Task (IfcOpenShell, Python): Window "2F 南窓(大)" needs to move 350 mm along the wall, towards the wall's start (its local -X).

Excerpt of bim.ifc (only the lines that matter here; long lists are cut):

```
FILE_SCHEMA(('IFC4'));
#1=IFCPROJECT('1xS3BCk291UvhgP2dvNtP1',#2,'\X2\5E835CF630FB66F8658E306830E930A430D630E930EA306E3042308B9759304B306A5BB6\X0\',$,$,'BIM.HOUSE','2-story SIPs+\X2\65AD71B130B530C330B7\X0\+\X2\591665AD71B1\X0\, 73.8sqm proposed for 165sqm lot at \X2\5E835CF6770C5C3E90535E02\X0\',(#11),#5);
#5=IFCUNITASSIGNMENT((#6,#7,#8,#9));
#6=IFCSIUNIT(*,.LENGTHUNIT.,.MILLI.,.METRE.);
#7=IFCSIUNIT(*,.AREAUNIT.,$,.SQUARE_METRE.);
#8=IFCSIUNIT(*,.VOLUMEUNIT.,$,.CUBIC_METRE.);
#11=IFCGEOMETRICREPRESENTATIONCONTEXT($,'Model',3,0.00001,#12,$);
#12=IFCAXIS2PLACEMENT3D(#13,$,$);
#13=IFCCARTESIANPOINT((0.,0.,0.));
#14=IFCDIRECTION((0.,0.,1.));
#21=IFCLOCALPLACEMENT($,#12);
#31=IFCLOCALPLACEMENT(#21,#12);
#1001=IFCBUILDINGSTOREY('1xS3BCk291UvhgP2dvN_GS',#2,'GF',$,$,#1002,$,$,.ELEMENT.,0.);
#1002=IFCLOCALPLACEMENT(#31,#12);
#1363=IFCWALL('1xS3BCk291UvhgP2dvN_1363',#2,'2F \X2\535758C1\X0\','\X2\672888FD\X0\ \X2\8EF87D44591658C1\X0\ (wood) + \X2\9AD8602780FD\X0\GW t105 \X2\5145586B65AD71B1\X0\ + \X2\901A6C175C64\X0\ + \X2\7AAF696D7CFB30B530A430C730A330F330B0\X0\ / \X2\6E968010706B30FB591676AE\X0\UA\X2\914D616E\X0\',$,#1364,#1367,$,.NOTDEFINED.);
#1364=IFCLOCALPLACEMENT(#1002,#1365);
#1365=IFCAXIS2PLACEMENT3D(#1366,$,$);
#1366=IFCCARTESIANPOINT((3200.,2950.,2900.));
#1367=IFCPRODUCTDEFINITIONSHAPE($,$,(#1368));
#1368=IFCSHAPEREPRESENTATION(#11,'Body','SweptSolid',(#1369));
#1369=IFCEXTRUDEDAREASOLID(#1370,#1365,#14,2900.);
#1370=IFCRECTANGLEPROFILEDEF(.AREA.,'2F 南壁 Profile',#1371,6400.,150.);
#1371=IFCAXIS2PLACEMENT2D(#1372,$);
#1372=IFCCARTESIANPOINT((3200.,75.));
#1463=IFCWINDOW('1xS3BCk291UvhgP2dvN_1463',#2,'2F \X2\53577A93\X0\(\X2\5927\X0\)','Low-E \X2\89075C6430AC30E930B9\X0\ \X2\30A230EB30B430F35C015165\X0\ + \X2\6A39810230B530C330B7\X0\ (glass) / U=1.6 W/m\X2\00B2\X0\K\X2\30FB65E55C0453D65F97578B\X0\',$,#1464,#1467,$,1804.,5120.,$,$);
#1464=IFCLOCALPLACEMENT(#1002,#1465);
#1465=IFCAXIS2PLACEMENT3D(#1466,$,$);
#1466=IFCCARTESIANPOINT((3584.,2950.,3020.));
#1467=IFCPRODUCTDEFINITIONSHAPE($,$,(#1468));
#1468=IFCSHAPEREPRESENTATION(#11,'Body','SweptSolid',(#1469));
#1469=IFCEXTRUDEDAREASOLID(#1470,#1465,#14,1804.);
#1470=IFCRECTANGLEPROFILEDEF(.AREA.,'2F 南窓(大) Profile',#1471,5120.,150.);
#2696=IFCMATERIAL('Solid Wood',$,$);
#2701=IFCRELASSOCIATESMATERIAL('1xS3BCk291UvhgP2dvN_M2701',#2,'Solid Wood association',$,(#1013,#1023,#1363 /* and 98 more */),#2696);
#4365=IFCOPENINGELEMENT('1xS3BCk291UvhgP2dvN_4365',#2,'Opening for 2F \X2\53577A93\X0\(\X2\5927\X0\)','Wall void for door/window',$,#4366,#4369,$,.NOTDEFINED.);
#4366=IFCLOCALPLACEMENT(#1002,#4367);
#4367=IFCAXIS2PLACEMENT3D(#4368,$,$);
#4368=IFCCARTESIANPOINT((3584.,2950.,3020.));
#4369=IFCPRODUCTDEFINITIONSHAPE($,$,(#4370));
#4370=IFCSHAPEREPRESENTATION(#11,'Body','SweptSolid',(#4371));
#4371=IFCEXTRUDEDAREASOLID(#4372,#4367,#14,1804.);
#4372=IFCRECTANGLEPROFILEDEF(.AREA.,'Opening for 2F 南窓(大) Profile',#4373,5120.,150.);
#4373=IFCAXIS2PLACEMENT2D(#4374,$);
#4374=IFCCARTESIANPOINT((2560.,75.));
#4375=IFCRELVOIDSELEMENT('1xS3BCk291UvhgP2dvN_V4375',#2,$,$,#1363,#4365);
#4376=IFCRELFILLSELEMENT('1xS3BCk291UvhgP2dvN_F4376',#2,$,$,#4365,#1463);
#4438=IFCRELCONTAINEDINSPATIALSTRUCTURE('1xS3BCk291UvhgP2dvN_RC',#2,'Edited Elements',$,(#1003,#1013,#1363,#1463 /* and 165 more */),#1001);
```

```python
import ifcopenshell
import ifcopenshell.api.geometry
import ifcopenshell.util.placement
import ifcopenshell.util.unit

model = ifcopenshell.open("bim.ifc")
unit_scale = ifcopenshell.util.unit.calculate_unit_scale(model)

window = model.by_id(1463)
opening = window.FillsVoids[0].RelatingOpeningElement
wall = opening.VoidsElements[0].RelatingBuildingElement

wall_matrix = ifcopenshell.util.placement.get_local_placement(wall.ObjectPlacement)
shift = wall_matrix[:3, 0] * -0.35 / unit_scale
before = ifcopenshell.util.placement.get_local_placement(window.ObjectPlacement)[:3, 3].copy()

# The window is not placed relative to its opening, so move both.
for product in (opening, window):
    matrix = ifcopenshell.util.placement.get_local_placement(product.ObjectPlacement)
    matrix[:3, 3] += shift
    ifcopenshell.api.geometry.edit_object_placement(model, product=product, matrix=matrix, is_si=False)

after = ifcopenshell.util.placement.get_local_placement(window.ObjectPlacement)[:3, 3]
print("window moved by", (after - before).round(3) + 0.0)

model.write("bim_rev.ifc")
```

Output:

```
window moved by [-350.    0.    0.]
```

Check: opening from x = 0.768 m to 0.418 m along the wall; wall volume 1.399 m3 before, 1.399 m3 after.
